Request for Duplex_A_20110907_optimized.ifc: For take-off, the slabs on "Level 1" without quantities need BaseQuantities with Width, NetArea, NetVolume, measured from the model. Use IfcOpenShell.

First a look at what the model holds.

```python
import ifcopenshell
import ifcopenshell.util.element
import ifcopenshell.util.unit

model = ifcopenshell.open("Duplex_A_20110907_optimized.ifc")
print(model.schema)
for unit_type in ("LENGTHUNIT", "AREAUNIT", "VOLUMEUNIT"):
    print(unit_type, ifcopenshell.util.unit.calculate_unit_scale(model, unit_type))
storey = next(s for s in model.by_type("IfcBuildingStorey") if s.Name == "Level 1")
slabs = [e for e in ifcopenshell.util.element.get_decomposition(storey) if e.is_a("IfcSlab")]
for e in sorted(slabs, key=lambda e: e.id()):
    print(e.id(), e.is_a(), e.Name, list(ifcopenshell.util.element.get_psets(e, qtos_only=True)), sep=" | ")
```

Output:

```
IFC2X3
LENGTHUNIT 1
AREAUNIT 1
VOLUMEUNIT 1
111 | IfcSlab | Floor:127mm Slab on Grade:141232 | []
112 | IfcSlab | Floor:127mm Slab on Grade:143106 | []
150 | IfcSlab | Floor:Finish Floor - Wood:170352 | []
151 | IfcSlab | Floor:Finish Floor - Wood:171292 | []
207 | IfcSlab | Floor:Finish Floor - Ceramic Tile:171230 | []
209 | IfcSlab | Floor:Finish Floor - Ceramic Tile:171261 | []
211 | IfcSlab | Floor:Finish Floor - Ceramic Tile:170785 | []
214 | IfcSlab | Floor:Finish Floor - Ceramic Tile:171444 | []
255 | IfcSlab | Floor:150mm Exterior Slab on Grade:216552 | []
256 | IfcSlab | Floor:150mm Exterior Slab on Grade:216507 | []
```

```python
import ifcopenshell
import ifcopenshell.api.pset
import ifcopenshell.geom
import ifcopenshell.util.element
import ifcopenshell.util.shape
import ifcopenshell.util.unit

model = ifcopenshell.open("Duplex_A_20110907_optimized.ifc")
unit_scale = ifcopenshell.util.unit.calculate_unit_scale(model)
area_scale = ifcopenshell.util.unit.calculate_unit_scale(model, "AREAUNIT")
volume_scale = ifcopenshell.util.unit.calculate_unit_scale(model, "VOLUMEUNIT")
settings = ifcopenshell.geom.settings()

storey = next(s for s in model.by_type("IfcBuildingStorey") if s.Name == "Level 1")
slabs = [e for e in ifcopenshell.util.element.get_decomposition(storey) if e.is_a("IfcSlab")]

for e in sorted(slabs, key=lambda e: e.id()):
    if ifcopenshell.util.element.get_psets(e, qtos_only=True, should_inherit=False):
        continue
    # Geometry comes back in metres, in the element's own axes.
    shape = ifcopenshell.geom.create_shape(settings, e)
    values = {
        "Width": ifcopenshell.util.shape.get_z(shape.geometry) / unit_scale,
        "NetArea": ifcopenshell.util.shape.get_footprint_area(shape.geometry) / area_scale,
        "NetVolume": ifcopenshell.util.shape.get_volume(shape.geometry) / volume_scale,
    }
    qto = ifcopenshell.api.pset.add_qto(model, product=e, name="BaseQuantities")
    ifcopenshell.api.pset.edit_qto(model, qto=qto, properties=values)
    print(e.id(), {k: round(v, 3) for k, v in values.items()})

model.write("Duplex_A_20110907_optimized_rev.ifc")
```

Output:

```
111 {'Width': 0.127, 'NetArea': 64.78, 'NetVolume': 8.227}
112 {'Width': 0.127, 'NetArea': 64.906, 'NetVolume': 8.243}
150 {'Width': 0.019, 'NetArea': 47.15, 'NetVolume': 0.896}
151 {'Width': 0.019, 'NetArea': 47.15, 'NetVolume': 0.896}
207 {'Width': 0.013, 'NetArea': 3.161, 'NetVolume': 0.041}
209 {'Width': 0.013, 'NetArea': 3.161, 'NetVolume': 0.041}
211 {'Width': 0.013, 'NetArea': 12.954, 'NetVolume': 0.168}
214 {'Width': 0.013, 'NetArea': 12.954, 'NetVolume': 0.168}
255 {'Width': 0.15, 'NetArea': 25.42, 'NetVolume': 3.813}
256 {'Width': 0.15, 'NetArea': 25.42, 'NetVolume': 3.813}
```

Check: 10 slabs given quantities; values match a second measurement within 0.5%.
